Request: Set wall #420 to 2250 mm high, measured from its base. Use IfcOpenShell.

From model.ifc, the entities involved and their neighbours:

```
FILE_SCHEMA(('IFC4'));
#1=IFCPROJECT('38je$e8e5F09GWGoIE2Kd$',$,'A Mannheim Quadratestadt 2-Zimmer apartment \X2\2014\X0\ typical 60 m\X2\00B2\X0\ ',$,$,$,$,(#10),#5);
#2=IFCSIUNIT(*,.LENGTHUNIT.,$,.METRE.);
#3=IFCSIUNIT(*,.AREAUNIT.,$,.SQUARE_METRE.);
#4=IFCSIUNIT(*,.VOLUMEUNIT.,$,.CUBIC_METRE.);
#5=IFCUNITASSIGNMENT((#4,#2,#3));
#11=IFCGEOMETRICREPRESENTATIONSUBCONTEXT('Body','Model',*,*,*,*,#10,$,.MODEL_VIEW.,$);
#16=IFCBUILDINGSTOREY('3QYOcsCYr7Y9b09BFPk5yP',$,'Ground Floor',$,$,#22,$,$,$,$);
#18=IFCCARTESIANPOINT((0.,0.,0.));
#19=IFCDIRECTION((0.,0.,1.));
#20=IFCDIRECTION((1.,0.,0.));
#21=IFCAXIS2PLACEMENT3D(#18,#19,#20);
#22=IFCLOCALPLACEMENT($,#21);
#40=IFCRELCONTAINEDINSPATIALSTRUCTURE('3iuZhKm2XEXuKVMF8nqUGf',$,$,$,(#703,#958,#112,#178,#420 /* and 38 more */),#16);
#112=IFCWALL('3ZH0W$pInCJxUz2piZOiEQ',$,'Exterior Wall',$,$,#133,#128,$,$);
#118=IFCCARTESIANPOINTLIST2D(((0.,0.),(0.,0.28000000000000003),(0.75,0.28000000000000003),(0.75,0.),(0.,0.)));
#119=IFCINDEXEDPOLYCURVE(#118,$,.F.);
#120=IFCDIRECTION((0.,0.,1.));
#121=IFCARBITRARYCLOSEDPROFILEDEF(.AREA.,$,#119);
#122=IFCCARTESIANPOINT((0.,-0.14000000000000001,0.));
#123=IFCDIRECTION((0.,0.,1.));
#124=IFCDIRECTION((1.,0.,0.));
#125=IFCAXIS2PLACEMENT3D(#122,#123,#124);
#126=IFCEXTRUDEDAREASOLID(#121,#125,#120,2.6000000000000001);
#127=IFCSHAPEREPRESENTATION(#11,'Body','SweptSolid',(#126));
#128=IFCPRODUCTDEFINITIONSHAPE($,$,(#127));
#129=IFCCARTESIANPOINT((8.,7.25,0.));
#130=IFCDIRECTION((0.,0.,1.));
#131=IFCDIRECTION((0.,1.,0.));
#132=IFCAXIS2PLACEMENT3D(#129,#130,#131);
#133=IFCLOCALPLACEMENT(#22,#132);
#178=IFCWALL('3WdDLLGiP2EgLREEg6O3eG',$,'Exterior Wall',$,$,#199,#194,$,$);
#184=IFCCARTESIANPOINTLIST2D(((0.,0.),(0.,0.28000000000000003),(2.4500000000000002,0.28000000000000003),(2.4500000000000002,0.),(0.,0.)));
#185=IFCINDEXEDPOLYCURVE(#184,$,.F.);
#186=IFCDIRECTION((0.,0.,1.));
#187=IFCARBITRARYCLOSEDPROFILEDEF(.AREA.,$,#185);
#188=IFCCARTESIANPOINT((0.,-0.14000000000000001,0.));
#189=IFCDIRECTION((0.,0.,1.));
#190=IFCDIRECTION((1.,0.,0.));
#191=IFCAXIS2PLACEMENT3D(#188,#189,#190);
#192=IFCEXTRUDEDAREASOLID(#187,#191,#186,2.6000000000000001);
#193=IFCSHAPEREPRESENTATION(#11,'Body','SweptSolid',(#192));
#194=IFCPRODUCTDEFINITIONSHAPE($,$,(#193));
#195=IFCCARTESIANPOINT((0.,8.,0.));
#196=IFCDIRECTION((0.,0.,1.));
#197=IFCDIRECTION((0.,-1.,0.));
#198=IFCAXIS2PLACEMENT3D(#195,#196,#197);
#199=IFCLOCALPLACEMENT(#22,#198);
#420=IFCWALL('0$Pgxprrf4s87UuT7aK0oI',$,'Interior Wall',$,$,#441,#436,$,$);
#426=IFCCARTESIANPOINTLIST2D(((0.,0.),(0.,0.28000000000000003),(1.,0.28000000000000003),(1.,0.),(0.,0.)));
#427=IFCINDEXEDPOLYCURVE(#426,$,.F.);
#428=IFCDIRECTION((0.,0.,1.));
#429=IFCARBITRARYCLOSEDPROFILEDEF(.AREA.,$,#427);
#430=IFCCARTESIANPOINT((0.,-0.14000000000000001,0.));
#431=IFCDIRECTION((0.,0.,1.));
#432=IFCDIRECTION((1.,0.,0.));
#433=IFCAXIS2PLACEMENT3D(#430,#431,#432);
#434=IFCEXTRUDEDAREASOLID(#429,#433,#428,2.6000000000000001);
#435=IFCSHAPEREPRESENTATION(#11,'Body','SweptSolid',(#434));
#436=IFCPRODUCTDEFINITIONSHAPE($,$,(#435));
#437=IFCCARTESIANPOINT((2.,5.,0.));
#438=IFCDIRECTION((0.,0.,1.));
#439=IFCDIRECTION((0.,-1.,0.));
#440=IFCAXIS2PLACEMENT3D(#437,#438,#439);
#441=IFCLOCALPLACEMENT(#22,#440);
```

```python
import ifcopenshell
import ifcopenshell.geom
import ifcopenshell.util.representation
import ifcopenshell.util.shape
import ifcopenshell.util.unit

model = ifcopenshell.open("model.ifc")
unit_scale = ifcopenshell.util.unit.calculate_unit_scale(model)
settings = ifcopenshell.geom.settings()


def volume(element):
    """Net volume in cubic metres, openings subtracted."""
    shape = ifcopenshell.geom.create_shape(settings, element)
    return ifcopenshell.util.shape.get_volume(shape.geometry)


wall = model.by_guid("0$Pgxprrf4s87UuT7aK0oI")
before = volume(wall)

body = ifcopenshell.util.representation.get_representation(wall, "Model", "Body")
solid = body.Items[0]
old_height = solid.Depth
solid.Depth = 2.25 / unit_scale
after = volume(wall)

print(f"height {old_height:g} -> {solid.Depth:g}, volume {before:.3f} -> {after:.3f} m3")

model.write("model_updated.ifc")
```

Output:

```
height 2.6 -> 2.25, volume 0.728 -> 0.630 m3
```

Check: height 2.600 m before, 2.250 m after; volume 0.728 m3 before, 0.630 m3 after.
